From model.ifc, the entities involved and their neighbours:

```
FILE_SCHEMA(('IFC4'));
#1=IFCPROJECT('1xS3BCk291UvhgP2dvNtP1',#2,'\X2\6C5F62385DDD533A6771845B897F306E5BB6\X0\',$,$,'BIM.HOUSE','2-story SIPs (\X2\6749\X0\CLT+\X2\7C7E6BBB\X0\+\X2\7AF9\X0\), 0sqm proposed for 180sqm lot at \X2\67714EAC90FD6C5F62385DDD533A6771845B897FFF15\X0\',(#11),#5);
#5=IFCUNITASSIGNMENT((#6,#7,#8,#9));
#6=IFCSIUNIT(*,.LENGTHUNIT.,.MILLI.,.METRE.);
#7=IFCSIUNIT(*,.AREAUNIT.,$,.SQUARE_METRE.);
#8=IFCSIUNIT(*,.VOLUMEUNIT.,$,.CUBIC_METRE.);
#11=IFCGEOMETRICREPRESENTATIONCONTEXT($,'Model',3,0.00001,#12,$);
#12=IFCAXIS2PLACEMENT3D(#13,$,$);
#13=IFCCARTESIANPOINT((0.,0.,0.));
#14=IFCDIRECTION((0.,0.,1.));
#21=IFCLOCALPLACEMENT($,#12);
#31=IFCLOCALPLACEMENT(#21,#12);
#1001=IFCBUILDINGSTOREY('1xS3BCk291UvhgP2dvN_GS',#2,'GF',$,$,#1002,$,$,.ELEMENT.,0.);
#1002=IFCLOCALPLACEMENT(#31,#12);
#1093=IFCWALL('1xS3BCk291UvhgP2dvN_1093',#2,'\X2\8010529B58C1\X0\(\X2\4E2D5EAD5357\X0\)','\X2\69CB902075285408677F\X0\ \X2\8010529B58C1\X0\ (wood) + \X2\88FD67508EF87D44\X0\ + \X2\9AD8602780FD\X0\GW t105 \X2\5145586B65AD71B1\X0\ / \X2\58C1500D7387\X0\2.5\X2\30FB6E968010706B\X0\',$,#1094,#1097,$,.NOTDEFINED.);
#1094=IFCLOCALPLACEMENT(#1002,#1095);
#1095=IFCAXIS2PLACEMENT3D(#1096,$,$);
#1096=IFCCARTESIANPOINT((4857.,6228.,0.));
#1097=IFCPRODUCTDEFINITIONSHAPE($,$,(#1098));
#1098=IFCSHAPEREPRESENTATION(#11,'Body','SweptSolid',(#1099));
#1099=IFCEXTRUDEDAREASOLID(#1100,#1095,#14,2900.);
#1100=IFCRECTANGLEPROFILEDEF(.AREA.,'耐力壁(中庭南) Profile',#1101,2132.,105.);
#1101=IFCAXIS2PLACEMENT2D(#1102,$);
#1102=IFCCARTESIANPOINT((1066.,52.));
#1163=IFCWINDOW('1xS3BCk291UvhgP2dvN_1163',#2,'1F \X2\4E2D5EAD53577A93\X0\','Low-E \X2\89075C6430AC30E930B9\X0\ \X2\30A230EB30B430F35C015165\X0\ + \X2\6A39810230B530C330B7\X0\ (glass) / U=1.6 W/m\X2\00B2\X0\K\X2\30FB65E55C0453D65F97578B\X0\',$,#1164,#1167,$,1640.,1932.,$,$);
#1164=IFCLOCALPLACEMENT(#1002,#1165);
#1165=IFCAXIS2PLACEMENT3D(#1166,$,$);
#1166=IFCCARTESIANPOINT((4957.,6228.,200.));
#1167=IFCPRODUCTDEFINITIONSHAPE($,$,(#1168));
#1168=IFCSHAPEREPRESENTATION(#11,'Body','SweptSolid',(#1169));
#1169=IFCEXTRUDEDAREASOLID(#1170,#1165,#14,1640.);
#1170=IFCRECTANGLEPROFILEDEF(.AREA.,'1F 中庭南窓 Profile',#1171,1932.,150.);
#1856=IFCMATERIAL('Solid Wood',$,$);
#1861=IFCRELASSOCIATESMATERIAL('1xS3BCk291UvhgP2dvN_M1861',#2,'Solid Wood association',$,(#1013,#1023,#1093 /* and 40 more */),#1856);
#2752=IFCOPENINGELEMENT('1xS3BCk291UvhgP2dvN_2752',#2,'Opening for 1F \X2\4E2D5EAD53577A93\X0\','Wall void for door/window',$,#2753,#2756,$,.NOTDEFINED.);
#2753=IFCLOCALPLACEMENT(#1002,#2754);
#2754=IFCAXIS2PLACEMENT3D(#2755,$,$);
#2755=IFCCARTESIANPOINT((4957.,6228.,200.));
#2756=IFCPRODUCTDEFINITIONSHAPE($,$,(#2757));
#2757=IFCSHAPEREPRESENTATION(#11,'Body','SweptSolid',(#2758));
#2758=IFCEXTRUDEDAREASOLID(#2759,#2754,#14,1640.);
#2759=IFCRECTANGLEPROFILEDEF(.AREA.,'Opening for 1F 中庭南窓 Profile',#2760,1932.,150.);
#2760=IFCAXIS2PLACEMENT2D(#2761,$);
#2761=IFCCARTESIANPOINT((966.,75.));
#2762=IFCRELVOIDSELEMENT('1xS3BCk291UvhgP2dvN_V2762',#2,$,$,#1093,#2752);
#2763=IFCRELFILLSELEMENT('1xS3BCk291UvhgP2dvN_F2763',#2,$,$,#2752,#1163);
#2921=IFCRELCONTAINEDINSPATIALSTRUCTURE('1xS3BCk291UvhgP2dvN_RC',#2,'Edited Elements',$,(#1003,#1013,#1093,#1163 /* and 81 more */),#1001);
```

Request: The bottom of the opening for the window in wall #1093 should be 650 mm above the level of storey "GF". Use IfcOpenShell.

```python
import numpy as np
import ifcopenshell
import ifcopenshell.api.geometry
import ifcopenshell.geom
import ifcopenshell.util.element
import ifcopenshell.util.placement
import ifcopenshell.util.shape
import ifcopenshell.util.unit

model = ifcopenshell.open("model.ifc")
unit_scale = ifcopenshell.util.unit.calculate_unit_scale(model)

window = model.by_id(1163)
opening = window.FillsVoids[0].RelatingOpeningElement
storey = ifcopenshell.util.element.get_container(window, ifc_class="IfcBuildingStorey")
level = ifcopenshell.util.placement.get_local_placement(storey.ObjectPlacement)[2, 3]

# The opening's origin need not be at the sill, so measure its lowest point.
shape = ifcopenshell.geom.create_shape(ifcopenshell.geom.settings(), opening)
bottom = ifcopenshell.util.shape.get_shape_bottom_elevation(shape, shape.geometry) / unit_scale
dz = level + 650.0 - bottom

shift = np.array([0.0, 0.0, dz])
# The window is not placed relative to its opening, so move both.
for product in (opening, window):
    matrix = ifcopenshell.util.placement.get_local_placement(product.ObjectPlacement)
    matrix[:3, 3] += shift
    ifcopenshell.api.geometry.edit_object_placement(model, product=product, matrix=matrix, is_si=False)

print(f"moved by {dz * unit_scale:+.3f} m")

model.write("model_updated.ifc")
```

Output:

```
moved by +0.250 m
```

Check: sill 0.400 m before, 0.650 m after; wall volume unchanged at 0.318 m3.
